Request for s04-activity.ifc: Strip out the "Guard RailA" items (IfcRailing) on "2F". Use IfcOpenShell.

First a look at what the model holds.

```python
import ifcopenshell
import ifcopenshell.util.element

model = ifcopenshell.open("s04-activity.ifc")
print(model.schema)
storey = next(s for s in model.by_type("IfcBuildingStorey") if s.Name == "2F")
railings = [e for e in ifcopenshell.util.element.get_decomposition(storey) if e.is_a("IfcRailing")]
seen = {}
for e in railings:
    element_type = ifcopenshell.util.element.get_type(e)
    name = element_type.Name if element_type not in (None, e) else None
    seen[name] = seen.get(name, 0) + 1
for name, count in sorted(seen.items(), key=str):
    print(count, "x", name)
```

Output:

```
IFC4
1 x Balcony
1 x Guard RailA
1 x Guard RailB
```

```python
import ifcopenshell
import ifcopenshell.api.root
import ifcopenshell.util.element

model = ifcopenshell.open("s04-activity.ifc")

storey = next(s for s in model.by_type("IfcBuildingStorey") if s.Name == "2F")
railings = [e for e in ifcopenshell.util.element.get_decomposition(storey) if e.is_a("IfcRailing")]
targets = [e for e in railings if (t := ifcopenshell.util.element.get_type(e)) not in (None, e) and t.Name == "Guard RailA"]

for e in targets:
    ifcopenshell.api.root.remove_product(model, product=e)
print(len(targets), "removed")

model.write("s04-activity_v2.ifc")
```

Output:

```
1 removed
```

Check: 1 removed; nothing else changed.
